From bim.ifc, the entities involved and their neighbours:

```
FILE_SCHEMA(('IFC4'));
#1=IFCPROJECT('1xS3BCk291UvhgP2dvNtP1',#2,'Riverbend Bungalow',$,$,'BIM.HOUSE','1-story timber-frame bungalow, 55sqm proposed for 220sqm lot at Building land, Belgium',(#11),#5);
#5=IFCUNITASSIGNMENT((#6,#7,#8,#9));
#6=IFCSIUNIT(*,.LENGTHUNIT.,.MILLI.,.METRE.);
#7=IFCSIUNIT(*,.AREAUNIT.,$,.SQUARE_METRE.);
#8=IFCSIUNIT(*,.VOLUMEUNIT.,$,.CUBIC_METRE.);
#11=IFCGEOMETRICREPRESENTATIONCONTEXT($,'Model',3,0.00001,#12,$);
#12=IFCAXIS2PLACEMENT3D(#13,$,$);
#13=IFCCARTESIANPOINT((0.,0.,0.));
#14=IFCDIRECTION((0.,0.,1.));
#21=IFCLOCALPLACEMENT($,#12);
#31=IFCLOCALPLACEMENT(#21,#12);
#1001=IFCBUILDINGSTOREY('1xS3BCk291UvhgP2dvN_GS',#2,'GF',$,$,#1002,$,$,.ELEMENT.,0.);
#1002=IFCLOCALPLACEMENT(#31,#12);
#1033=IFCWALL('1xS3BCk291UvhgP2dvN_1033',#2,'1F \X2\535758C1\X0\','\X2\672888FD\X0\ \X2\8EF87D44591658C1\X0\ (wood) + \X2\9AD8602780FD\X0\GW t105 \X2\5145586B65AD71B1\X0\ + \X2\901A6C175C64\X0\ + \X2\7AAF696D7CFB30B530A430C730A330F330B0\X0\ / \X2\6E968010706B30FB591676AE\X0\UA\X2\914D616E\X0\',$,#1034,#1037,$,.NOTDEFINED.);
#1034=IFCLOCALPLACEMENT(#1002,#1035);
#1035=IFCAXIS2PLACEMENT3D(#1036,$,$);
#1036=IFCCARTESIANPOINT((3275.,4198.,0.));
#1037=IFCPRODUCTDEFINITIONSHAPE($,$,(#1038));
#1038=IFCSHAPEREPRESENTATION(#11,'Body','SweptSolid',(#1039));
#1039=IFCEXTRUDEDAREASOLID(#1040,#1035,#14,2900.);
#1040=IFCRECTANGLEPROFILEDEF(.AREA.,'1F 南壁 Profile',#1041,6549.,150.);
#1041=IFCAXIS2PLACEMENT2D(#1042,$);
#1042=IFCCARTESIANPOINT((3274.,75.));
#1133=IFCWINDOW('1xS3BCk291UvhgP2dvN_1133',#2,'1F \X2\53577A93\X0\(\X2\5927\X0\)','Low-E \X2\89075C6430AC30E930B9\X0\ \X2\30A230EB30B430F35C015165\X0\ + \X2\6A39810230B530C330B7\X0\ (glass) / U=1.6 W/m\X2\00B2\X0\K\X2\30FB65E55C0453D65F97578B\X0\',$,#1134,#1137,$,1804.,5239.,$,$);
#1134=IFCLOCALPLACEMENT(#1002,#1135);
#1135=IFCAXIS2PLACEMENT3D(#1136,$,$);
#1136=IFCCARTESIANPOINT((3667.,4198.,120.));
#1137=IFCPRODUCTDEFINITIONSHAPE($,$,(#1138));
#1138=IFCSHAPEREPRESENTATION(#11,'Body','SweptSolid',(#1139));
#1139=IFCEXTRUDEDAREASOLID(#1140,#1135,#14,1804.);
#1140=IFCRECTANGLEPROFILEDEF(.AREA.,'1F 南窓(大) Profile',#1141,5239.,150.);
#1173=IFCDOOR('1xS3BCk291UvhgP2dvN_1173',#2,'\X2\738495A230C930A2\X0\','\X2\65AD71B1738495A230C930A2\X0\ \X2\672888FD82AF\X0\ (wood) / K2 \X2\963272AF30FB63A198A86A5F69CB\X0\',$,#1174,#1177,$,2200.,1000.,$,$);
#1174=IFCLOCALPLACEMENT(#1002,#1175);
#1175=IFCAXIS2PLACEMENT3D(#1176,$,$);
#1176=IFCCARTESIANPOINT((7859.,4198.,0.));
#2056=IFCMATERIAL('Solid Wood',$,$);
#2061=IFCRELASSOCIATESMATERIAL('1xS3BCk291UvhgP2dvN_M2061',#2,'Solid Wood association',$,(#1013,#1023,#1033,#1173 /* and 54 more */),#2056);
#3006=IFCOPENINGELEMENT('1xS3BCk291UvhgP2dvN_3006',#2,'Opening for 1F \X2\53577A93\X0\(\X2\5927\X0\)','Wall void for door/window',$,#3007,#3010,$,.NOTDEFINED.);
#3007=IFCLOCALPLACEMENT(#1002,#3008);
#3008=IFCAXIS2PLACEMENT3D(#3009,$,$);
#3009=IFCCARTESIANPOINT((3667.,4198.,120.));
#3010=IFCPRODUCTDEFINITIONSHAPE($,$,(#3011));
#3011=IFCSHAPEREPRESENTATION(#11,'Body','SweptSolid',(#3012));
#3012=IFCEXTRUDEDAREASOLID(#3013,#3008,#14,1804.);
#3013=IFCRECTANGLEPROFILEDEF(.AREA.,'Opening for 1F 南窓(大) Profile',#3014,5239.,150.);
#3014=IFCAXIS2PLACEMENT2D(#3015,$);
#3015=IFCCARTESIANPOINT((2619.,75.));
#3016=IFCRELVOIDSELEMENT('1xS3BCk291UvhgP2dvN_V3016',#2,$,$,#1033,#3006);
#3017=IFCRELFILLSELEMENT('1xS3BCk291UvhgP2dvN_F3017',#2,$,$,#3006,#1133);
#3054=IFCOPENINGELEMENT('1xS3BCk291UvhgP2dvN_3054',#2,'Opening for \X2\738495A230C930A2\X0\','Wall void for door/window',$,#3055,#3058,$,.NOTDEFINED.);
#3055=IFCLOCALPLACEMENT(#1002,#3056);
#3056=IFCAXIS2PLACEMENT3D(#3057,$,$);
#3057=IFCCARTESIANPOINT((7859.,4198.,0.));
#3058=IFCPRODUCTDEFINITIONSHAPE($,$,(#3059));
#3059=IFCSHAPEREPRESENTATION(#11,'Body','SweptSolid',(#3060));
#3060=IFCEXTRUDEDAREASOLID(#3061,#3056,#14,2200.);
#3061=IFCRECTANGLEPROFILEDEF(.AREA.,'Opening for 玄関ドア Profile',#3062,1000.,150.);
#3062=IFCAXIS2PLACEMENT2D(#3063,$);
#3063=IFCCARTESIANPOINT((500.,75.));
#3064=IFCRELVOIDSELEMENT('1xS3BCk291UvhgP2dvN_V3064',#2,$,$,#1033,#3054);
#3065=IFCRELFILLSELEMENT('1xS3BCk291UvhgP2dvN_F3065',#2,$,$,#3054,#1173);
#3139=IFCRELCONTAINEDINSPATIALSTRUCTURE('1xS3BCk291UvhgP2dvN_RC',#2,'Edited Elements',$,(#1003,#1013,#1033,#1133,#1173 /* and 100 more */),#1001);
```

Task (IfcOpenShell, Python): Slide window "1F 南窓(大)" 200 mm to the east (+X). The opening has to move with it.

```python
import ifcopenshell
import ifcopenshell.api.geometry
import ifcopenshell.util.placement

model = ifcopenshell.open("bim.ifc")

window = model.by_guid("1xS3BCk291UvhgP2dvN_1133")
opening = window.FillsVoids[0].RelatingOpeningElement
wall = opening.VoidsElements[0].RelatingBuildingElement

wall_matrix = ifcopenshell.util.placement.get_local_placement(wall.ObjectPlacement)
shift = wall_matrix[:3, 0] * 200.0
before = ifcopenshell.util.placement.get_local_placement(window.ObjectPlacement)[:3, 3].copy()

# The window is not placed relative to its opening, so move both.
for product in (opening, window):
    matrix = ifcopenshell.util.placement.get_local_placement(product.ObjectPlacement)
    matrix[:3, 3] += shift
    ifcopenshell.api.geometry.edit_object_placement(model, product=product, matrix=matrix, is_si=False)

after = ifcopenshell.util.placement.get_local_placement(window.ObjectPlacement)[:3, 3]
print("window moved by", (after - before).round(3) + 0.0)

model.write("bim_updated.ifc")
```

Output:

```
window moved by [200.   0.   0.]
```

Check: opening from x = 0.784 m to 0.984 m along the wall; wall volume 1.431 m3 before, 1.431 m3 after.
